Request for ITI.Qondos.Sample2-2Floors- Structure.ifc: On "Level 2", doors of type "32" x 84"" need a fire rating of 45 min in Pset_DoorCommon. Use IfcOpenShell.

First a look at what the model holds.

```python
import ifcopenshell
import ifcopenshell.util.element

model = ifcopenshell.open("ITI.Qondos.Sample2-2Floors- Structure.ifc")
print(model.schema)
storey = next(s for s in model.by_type("IfcBuildingStorey") if s.Name == "Level 2")
doors = [e for e in ifcopenshell.util.element.get_decomposition(storey) if e.is_a("IfcDoor")]
seen = {}
for e in doors:
    element_type = ifcopenshell.util.element.get_type(e)
    key = (element_type.Name if element_type != e and element_type else None, ifcopenshell.util.element.get_pset(e, "Pset_DoorCommon", "FireRating"))
    seen[key] = seen.get(key, 0) + 1
for (name, value), count in sorted(seen.items(), key=str):
    print(count, "x", name, "|", value)
```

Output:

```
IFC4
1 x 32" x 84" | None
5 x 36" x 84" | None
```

```python
import ifcopenshell
import ifcopenshell.api.pset
import ifcopenshell.util.element

model = ifcopenshell.open("ITI.Qondos.Sample2-2Floors- Structure.ifc")

storey = next(s for s in model.by_type("IfcBuildingStorey") if s.Name == "Level 2")
doors = [e for e in ifcopenshell.util.element.get_decomposition(storey) if e.is_a("IfcDoor")]

count = 0
for e in doors:
    element_type = ifcopenshell.util.element.get_type(e)
    if element_type in (None, e) or element_type.Name != '32" x 84"':
        continue
    # add_pset returns the element's existing set when there is one.
    pset = ifcopenshell.api.pset.add_pset(model, product=e, name="Pset_DoorCommon")
    ifcopenshell.api.pset.edit_pset(model, pset=pset, properties={"FireRating": "45 min"})
    count += 1

print(count, "doors updated")

model.write("ITI.Qondos.Sample2-2Floors- Structure_rev.ifc")
```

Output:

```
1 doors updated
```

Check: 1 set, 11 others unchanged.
